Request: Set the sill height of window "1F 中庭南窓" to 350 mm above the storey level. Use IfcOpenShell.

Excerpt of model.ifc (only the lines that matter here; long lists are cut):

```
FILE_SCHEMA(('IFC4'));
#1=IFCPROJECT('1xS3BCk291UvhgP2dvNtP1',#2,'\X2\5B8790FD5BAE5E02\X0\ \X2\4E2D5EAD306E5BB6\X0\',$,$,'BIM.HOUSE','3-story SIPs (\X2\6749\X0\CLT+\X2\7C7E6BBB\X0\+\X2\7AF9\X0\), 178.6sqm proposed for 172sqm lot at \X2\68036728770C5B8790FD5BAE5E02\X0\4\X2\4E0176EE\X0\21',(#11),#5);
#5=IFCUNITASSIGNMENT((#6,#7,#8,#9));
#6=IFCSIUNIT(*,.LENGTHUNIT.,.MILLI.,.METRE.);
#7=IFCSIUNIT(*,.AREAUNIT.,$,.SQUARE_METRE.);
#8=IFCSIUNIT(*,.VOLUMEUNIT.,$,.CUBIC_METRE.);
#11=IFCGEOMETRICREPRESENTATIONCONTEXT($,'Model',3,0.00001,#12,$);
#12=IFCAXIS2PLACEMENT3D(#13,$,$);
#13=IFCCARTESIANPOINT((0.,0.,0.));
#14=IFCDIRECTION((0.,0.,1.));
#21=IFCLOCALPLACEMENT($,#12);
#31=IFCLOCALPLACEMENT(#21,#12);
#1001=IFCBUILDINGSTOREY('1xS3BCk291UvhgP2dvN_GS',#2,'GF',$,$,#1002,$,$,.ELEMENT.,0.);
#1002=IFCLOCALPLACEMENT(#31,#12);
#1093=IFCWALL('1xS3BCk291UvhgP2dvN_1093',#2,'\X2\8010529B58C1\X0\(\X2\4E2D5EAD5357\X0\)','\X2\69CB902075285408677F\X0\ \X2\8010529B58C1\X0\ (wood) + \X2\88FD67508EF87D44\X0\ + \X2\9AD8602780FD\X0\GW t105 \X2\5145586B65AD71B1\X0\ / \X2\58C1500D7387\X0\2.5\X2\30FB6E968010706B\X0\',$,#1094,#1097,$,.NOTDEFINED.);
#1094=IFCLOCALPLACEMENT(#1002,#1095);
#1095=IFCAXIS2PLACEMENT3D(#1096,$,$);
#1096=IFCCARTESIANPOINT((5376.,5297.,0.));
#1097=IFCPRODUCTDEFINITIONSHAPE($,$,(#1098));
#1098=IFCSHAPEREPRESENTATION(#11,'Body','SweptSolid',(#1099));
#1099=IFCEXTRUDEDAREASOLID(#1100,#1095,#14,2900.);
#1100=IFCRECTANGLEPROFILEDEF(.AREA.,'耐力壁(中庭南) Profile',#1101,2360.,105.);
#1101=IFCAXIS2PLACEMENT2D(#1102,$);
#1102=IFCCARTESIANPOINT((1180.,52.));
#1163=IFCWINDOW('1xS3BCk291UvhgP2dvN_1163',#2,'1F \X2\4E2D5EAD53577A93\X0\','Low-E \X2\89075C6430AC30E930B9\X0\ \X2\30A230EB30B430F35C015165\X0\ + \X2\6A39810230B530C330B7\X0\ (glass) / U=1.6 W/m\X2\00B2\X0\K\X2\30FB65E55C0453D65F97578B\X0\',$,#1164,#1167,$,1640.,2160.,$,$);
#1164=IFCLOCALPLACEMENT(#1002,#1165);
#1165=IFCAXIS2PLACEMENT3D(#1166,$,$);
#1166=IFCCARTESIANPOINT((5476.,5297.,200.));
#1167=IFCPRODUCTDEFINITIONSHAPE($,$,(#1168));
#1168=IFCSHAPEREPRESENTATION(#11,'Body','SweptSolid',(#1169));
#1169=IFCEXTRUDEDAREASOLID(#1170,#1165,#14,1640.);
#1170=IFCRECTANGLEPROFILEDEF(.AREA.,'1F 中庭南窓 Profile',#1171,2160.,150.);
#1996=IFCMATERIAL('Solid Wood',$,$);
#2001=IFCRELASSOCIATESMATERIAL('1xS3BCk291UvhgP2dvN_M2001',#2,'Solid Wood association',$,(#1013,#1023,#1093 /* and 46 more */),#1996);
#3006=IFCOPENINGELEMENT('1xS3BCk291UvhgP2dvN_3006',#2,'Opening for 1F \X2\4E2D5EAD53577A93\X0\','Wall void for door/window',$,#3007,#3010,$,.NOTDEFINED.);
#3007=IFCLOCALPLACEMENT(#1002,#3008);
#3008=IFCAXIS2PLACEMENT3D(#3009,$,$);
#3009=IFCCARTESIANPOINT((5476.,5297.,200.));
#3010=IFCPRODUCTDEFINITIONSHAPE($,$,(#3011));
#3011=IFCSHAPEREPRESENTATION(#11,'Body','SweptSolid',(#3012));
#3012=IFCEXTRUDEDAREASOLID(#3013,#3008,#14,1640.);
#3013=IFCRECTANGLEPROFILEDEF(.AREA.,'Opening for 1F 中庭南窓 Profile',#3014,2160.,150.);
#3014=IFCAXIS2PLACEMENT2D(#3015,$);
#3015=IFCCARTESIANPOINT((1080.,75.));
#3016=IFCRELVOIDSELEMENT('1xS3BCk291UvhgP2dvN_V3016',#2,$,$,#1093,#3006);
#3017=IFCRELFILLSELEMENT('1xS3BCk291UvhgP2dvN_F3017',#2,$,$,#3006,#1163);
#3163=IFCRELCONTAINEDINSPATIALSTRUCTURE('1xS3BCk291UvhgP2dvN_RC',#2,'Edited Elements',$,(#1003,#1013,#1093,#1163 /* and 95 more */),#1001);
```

```python
import numpy as np
import ifcopenshell
import ifcopenshell.api.geometry
import ifcopenshell.geom
import ifcopenshell.util.element
import ifcopenshell.util.placement
import ifcopenshell.util.shape
import ifcopenshell.util.unit

model = ifcopenshell.open("model.ifc")
unit_scale = ifcopenshell.util.unit.calculate_unit_scale(model)

window = model.by_guid("1xS3BCk291UvhgP2dvN_1163")
opening = window.FillsVoids[0].RelatingOpeningElement
storey = ifcopenshell.util.element.get_container(window, ifc_class="IfcBuildingStorey")
level = ifcopenshell.util.placement.get_local_placement(storey.ObjectPlacement)[2, 3]

# The opening's origin need not be at the sill, so measure its lowest point.
shape = ifcopenshell.geom.create_shape(ifcopenshell.geom.settings(), opening)
bottom = ifcopenshell.util.shape.get_shape_bottom_elevation(shape, shape.geometry) / unit_scale
dz = level + 350.0 - bottom

shift = np.array([0.0, 0.0, dz])
# The window is not placed relative to its opening, so move both.
for product in (opening, window):
    matrix = ifcopenshell.util.placement.get_local_placement(product.ObjectPlacement)
    matrix[:3, 3] += shift
    ifcopenshell.api.geometry.edit_object_placement(model, product=product, matrix=matrix, is_si=False)

print(f"moved by {dz * unit_scale:+.3f} m")

model.write("model_edited.ifc")
```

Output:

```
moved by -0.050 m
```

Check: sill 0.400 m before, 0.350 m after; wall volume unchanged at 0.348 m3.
